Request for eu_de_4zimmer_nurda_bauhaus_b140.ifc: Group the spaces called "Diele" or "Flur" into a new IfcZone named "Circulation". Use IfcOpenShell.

First a look at what the model holds.

```python
import ifcopenshell

model = ifcopenshell.open("eu_de_4zimmer_nurda_bauhaus_b140.ifc")
print(model.schema)
seen = {}
for space in model.by_type("IfcSpace"):
    seen[space.LongName] = seen.get(space.LongName, 0) + 1
for name, count in sorted(seen.items(), key=str):
    print(count, "x", name)
print("zones:", [z.Name for z in model.by_type("IfcZone")][:20])
```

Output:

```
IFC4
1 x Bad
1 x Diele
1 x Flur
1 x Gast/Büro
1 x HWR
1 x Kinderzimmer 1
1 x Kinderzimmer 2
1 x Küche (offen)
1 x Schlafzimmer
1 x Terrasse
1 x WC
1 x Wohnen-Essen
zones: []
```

```python
import ifcopenshell
import ifcopenshell.api.group
import ifcopenshell.api.root

model = ifcopenshell.open("eu_de_4zimmer_nurda_bauhaus_b140.ifc")

names = {"Diele", "Flur"}
spaces = [s for s in model.by_type("IfcSpace") if s.LongName in names]

zone = ifcopenshell.api.root.create_entity(model, ifc_class="IfcZone", name="Circulation")
ifcopenshell.api.group.assign_group(model, products=spaces, group=zone)
print(len(spaces), "spaces in", zone.Name)

model.write("eu_de_4zimmer_nurda_bauhaus_b140_v2.ifc")
```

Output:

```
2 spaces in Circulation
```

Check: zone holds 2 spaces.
